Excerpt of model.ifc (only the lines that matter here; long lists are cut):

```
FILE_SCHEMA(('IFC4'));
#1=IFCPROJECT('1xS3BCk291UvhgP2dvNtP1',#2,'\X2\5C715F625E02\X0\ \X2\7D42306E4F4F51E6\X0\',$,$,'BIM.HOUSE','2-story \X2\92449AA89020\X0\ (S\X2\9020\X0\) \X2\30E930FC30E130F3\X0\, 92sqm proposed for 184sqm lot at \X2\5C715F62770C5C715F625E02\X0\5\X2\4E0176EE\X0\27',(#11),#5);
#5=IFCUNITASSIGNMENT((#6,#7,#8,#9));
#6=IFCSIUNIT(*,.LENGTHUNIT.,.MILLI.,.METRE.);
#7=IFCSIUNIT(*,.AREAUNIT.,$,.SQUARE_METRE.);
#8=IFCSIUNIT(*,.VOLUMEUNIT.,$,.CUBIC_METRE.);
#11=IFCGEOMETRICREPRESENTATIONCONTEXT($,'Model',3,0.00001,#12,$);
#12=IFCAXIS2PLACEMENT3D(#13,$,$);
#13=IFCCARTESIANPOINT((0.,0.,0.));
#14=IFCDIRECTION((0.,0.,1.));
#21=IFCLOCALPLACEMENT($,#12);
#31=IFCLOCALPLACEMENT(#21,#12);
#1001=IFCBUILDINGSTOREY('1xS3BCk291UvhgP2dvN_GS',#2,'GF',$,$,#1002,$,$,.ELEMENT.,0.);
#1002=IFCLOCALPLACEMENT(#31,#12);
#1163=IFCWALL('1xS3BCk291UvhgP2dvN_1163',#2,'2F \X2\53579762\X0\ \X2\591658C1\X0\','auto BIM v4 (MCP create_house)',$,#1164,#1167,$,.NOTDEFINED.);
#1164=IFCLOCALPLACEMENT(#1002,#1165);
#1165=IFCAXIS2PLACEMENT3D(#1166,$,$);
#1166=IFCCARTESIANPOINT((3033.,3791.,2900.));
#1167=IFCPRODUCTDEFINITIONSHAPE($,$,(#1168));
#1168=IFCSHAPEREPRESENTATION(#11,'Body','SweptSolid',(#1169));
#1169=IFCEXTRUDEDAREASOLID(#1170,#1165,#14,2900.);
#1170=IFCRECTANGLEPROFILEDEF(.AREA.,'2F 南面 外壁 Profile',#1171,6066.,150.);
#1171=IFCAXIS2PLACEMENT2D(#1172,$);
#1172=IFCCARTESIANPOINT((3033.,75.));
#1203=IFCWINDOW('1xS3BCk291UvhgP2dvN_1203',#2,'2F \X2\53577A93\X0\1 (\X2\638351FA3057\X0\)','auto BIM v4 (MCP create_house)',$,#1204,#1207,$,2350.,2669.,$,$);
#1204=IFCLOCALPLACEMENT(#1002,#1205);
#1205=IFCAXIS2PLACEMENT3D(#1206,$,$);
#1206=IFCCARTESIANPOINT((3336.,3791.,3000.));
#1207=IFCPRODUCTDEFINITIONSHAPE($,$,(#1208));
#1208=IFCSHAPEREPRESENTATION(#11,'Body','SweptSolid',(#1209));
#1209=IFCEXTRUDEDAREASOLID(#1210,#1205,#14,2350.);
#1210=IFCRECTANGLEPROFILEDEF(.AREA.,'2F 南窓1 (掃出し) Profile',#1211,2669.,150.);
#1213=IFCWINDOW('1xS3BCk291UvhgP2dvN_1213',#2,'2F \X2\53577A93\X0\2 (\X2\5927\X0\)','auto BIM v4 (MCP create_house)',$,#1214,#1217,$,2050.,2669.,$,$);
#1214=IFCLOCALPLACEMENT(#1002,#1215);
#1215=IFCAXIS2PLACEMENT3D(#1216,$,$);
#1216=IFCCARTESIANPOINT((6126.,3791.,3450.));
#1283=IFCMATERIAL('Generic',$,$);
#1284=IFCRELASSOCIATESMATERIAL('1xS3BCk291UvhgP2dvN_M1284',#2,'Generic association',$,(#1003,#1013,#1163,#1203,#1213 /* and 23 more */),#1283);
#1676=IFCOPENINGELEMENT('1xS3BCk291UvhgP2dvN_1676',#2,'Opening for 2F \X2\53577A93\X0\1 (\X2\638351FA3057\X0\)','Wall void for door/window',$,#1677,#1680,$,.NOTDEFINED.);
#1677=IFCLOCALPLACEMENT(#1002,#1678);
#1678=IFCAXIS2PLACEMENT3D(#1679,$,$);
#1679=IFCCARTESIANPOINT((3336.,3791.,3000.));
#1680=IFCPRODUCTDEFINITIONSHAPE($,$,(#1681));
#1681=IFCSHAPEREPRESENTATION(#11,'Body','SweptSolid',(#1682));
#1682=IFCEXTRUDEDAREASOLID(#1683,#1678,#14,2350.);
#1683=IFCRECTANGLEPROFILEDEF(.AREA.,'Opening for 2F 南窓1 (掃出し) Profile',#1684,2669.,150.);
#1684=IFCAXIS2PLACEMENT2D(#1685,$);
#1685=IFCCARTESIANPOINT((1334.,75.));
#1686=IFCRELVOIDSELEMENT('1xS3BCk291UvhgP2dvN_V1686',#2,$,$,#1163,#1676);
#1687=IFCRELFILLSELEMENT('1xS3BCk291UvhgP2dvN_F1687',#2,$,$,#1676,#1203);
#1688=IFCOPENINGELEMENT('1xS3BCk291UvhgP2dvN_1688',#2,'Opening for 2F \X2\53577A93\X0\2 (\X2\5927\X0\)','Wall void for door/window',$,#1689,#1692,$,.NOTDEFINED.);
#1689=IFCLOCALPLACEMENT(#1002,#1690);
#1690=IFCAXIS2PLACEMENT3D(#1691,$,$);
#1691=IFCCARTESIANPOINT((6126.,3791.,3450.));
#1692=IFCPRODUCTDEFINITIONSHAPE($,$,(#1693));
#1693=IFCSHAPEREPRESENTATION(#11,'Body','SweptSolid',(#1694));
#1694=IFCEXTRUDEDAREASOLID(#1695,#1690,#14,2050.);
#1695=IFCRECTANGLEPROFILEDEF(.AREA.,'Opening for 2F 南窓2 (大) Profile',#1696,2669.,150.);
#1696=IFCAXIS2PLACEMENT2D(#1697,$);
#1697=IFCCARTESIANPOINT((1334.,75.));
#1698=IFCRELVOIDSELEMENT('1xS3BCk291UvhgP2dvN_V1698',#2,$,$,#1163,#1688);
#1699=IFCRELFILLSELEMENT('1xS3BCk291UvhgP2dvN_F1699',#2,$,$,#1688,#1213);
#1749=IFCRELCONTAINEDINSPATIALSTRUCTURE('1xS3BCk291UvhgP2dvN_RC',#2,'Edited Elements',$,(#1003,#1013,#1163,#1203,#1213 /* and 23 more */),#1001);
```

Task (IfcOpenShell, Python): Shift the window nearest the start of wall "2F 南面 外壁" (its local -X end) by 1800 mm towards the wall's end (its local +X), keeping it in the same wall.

```python
import ifcopenshell
import ifcopenshell.api.geometry
import ifcopenshell.util.placement
import ifcopenshell.util.unit

model = ifcopenshell.open("model.ifc")
unit_scale = ifcopenshell.util.unit.calculate_unit_scale(model)

window = model.by_guid("1xS3BCk291UvhgP2dvN_1203")
opening = window.FillsVoids[0].RelatingOpeningElement
wall = opening.VoidsElements[0].RelatingBuildingElement

wall_matrix = ifcopenshell.util.placement.get_local_placement(wall.ObjectPlacement)
shift = wall_matrix[:3, 0] * 1.8 / unit_scale
before = ifcopenshell.util.placement.get_local_placement(window.ObjectPlacement)[:3, 3].copy()

# The window is not placed relative to its opening, so move both.
for product in (opening, window):
    matrix = ifcopenshell.util.placement.get_local_placement(product.ObjectPlacement)
    matrix[:3, 3] += shift
    ifcopenshell.api.geometry.edit_object_placement(model, product=product, matrix=matrix, is_si=False)

after = ifcopenshell.util.placement.get_local_placement(window.ObjectPlacement)[:3, 3]
print("window moved by", (after - before).round(3) + 0.0)

model.write("model_updated.ifc")
```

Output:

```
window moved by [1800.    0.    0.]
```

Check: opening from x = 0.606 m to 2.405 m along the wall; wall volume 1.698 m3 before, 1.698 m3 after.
